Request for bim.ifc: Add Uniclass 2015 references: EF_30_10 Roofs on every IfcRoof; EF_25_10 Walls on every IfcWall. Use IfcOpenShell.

First a look at what the model holds.

```python
import ifcopenshell

model = ifcopenshell.open("bim.ifc")
print(model.schema)
print("classifications:", [c.Name for c in model.by_type("IfcClassification")])
for ifc_class in ("IfcDoor", "IfcRoof", "IfcStair", "IfcWall", "IfcWindow"):
    print(ifc_class, len(model.by_type(ifc_class)))
```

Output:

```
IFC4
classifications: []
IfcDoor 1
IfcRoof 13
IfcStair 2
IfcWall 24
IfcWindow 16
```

```python
import ifcopenshell
import ifcopenshell.api.classification

model = ifcopenshell.open("bim.ifc")

system = ifcopenshell.api.classification.add_classification(model, classification="Uniclass 2015")

codes = {
    "IfcRoof": ("EF_30_10", "Roofs"),
    "IfcWall": ("EF_25_10", "Walls"),
}
for ifc_class, (code, name) in codes.items():
    products = model.by_type(ifc_class)
    ifcopenshell.api.classification.add_reference(
        model, products=products, classification=system, identification=code, name=name
    )
    print(code, len(products))

model.write("bim-out.ifc")
```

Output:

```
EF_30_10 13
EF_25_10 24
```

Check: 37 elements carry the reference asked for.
